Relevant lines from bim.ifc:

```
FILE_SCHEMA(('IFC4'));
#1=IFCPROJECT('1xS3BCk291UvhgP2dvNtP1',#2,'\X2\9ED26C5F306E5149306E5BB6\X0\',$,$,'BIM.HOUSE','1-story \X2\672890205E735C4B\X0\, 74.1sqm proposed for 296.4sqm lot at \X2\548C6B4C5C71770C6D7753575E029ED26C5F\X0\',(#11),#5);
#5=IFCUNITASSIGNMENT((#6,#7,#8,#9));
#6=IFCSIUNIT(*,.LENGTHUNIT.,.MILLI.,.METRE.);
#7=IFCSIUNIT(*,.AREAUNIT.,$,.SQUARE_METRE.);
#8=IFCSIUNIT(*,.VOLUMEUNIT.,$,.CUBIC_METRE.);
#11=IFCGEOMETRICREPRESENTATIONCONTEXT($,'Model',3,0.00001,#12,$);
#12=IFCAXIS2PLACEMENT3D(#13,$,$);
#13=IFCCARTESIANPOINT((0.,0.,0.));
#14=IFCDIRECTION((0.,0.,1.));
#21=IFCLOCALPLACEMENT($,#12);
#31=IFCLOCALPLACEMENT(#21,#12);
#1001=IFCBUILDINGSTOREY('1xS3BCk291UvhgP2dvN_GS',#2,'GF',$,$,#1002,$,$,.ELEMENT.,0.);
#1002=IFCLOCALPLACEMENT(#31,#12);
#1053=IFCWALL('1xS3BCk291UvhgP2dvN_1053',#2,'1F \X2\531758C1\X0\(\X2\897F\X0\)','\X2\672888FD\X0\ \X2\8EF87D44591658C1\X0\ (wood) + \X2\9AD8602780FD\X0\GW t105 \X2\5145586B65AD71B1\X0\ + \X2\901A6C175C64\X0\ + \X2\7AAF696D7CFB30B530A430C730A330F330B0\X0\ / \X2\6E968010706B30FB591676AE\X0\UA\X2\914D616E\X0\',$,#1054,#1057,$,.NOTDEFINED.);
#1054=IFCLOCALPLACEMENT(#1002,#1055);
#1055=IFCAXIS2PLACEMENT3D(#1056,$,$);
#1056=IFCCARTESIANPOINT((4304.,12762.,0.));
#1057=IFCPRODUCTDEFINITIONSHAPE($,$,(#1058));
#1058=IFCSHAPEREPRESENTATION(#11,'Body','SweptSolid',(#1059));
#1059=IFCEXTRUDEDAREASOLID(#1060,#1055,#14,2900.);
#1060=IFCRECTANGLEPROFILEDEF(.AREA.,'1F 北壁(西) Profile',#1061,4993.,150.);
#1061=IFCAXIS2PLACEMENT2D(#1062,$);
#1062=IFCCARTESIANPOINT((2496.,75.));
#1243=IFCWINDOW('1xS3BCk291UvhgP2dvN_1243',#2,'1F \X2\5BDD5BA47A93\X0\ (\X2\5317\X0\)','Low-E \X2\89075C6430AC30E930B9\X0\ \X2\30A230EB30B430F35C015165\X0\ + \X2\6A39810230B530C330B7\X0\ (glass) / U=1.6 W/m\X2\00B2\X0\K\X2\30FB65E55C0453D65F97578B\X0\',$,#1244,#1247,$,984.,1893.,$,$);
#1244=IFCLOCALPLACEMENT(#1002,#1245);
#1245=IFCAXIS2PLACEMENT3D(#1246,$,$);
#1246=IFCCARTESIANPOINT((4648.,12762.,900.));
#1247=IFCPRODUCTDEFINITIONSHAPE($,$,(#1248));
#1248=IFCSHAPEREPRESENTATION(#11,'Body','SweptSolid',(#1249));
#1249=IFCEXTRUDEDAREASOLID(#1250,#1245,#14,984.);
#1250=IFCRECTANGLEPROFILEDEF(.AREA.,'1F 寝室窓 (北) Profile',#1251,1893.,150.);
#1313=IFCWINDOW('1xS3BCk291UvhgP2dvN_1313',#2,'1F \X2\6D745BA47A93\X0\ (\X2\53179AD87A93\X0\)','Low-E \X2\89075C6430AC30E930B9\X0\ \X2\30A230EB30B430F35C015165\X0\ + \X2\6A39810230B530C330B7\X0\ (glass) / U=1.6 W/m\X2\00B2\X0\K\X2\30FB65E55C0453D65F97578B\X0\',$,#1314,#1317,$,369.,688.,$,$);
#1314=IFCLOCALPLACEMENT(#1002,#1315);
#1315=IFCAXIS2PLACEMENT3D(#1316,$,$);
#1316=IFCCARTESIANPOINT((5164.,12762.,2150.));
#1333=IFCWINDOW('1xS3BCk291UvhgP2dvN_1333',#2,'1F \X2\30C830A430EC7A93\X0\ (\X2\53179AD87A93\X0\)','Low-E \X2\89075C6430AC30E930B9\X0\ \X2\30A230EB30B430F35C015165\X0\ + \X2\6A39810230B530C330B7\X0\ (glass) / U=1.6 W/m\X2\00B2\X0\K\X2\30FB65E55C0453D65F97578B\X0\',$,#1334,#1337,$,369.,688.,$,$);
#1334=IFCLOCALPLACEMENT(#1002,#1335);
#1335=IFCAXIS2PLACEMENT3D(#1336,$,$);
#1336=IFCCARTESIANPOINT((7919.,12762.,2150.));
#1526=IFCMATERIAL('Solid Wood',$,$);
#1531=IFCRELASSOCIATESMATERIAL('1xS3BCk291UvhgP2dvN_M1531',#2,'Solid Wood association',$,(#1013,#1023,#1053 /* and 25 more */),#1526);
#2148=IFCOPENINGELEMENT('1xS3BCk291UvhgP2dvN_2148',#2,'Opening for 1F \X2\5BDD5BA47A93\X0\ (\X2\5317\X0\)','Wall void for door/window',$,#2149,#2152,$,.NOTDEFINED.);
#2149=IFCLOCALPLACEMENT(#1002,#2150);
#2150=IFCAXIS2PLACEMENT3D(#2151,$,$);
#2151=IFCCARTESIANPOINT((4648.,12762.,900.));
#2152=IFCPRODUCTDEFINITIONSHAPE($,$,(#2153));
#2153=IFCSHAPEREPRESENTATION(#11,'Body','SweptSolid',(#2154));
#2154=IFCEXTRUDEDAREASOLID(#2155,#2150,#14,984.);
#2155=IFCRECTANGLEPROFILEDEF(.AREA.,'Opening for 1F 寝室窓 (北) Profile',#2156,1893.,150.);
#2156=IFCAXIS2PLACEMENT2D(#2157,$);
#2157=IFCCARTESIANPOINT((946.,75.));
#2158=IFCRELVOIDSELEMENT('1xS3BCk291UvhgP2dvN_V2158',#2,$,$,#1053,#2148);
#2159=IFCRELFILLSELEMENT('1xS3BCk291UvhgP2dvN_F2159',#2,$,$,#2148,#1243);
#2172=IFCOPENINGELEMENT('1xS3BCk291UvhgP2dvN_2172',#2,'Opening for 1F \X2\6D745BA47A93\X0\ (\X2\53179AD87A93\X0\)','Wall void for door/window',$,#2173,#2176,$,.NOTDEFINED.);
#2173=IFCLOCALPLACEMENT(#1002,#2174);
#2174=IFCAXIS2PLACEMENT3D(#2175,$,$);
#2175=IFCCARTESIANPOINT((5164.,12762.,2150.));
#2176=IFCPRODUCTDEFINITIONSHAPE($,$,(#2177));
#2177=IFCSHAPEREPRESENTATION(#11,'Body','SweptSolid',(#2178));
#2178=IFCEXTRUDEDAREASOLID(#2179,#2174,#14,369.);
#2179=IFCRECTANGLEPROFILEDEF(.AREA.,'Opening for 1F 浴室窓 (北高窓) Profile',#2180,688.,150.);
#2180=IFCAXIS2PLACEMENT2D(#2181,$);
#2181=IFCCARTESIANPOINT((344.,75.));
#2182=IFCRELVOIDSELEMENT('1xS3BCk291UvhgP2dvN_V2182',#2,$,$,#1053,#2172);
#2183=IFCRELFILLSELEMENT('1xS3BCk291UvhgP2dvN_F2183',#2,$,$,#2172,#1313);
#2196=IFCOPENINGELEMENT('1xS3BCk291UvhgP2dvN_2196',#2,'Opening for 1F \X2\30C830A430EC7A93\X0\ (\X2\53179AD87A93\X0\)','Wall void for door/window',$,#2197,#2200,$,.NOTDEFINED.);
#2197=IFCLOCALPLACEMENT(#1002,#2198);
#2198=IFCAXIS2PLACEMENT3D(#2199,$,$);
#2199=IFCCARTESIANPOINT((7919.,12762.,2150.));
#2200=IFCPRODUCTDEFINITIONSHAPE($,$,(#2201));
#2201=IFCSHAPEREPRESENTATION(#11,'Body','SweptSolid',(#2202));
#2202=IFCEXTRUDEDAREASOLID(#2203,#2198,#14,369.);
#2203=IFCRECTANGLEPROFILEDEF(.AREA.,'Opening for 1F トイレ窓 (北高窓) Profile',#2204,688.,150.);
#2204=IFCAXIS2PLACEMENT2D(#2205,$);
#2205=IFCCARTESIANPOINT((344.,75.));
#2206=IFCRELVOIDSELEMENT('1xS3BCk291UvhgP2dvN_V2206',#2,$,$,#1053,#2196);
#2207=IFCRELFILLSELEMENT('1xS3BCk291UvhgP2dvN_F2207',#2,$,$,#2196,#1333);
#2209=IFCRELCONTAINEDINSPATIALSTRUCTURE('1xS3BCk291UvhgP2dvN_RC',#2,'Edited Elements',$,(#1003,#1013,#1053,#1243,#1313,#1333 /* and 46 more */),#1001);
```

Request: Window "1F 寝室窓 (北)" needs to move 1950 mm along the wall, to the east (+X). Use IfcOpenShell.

```python
import ifcopenshell
import ifcopenshell.api.geometry
import ifcopenshell.util.placement
import ifcopenshell.util.unit

model = ifcopenshell.open("bim.ifc")
unit_scale = ifcopenshell.util.unit.calculate_unit_scale(model)

window = model.by_guid("1xS3BCk291UvhgP2dvN_1243")
opening = window.FillsVoids[0].RelatingOpeningElement
wall = opening.VoidsElements[0].RelatingBuildingElement

wall_matrix = ifcopenshell.util.placement.get_local_placement(wall.ObjectPlacement)
shift = wall_matrix[:3, 0] * 1.95 / unit_scale
before = ifcopenshell.util.placement.get_local_placement(window.ObjectPlacement)[:3, 3].copy()

# The window is not placed relative to its opening, so move both.
for product in (opening, window):
    matrix = ifcopenshell.util.placement.get_local_placement(product.ObjectPlacement)
    matrix[:3, 3] += shift
    ifcopenshell.api.geometry.edit_object_placement(model, product=product, matrix=matrix, is_si=False)

after = ifcopenshell.util.placement.get_local_placement(window.ObjectPlacement)[:3, 3]
print("window moved by", (after - before).round(3) + 0.0)

model.write("bim_edited.ifc")
```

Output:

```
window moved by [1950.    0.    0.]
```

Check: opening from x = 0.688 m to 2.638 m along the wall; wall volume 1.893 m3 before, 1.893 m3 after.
